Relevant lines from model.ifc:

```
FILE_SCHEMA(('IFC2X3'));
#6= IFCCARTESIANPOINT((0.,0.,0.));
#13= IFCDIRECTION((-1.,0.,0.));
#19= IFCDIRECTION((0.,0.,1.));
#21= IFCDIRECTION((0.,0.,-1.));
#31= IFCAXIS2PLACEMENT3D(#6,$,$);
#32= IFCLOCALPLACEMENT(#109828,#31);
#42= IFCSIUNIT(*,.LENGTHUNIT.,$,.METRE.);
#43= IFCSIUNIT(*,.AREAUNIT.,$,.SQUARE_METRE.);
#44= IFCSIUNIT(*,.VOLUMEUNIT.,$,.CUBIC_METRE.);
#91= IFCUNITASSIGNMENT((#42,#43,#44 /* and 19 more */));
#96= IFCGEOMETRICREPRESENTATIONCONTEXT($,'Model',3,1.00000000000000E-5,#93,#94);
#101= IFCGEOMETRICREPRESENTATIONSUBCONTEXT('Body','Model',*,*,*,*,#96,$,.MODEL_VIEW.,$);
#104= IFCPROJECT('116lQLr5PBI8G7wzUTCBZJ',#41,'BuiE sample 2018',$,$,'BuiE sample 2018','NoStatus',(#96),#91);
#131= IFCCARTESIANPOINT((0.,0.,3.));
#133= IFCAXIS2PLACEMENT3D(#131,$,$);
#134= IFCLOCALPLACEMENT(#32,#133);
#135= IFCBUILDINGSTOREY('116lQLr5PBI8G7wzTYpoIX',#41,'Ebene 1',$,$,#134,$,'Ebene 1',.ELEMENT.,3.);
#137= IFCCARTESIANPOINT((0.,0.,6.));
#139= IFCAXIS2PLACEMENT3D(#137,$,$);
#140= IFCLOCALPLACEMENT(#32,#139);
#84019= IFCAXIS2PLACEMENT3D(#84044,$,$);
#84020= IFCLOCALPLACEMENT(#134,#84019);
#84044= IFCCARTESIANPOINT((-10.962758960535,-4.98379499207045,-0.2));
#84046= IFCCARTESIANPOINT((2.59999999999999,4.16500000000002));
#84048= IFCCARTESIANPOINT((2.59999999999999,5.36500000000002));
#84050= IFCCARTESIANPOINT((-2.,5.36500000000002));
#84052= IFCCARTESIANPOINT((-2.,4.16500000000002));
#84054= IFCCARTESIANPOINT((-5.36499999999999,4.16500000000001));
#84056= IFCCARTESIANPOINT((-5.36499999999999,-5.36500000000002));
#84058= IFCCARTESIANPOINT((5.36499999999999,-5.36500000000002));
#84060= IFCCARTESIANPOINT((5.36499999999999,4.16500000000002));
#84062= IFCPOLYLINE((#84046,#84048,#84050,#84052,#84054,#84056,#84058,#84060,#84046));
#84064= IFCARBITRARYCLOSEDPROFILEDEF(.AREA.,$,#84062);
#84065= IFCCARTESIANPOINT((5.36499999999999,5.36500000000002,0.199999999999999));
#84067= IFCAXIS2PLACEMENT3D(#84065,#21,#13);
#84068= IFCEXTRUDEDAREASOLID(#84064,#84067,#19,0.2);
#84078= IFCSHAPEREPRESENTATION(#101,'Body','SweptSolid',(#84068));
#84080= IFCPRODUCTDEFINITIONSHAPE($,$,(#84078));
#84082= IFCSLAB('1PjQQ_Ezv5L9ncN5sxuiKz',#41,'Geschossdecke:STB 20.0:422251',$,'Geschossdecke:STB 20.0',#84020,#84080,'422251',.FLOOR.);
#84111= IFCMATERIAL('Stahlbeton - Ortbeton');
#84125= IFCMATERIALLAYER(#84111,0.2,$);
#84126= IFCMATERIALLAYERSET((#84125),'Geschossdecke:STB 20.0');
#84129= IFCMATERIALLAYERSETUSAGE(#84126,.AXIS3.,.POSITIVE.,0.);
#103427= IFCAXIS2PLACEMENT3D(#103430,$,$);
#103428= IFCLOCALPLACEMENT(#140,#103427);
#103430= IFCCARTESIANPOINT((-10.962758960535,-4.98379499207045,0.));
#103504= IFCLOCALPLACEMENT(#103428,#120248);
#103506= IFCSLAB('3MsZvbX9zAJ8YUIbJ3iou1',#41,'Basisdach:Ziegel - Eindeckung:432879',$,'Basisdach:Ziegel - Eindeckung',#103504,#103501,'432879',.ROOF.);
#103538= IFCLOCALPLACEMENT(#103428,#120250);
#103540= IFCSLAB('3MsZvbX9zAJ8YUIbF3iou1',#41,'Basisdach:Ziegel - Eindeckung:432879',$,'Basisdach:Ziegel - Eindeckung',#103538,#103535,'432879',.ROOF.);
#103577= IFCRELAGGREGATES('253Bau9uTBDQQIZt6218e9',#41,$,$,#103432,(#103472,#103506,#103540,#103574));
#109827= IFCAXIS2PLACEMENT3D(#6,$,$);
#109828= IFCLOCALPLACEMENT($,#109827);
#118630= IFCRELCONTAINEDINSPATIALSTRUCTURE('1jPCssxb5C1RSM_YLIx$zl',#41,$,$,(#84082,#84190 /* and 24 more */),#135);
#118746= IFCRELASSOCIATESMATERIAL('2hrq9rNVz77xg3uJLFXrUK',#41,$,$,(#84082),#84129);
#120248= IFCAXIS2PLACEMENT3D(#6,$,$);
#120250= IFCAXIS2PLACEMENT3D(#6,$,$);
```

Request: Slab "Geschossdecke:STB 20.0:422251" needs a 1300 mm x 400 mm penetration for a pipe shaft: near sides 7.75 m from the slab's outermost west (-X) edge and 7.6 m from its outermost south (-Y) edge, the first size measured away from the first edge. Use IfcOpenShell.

```python
import numpy as np
import ifcopenshell
import ifcopenshell.api.feature
import ifcopenshell.api.geometry
import ifcopenshell.api.root
import ifcopenshell.geom
import ifcopenshell.util.placement
import ifcopenshell.util.representation
import ifcopenshell.util.shape
import ifcopenshell.util.unit

model = ifcopenshell.open("model.ifc")
unit_scale = ifcopenshell.util.unit.calculate_unit_scale(model)
settings = ifcopenshell.geom.settings()


def volume(element):
    """Net volume in cubic metres, openings subtracted."""
    shape = ifcopenshell.geom.create_shape(settings, element)
    return ifcopenshell.util.shape.get_volume(shape.geometry)


slab = model.by_id(84082)
before = volume(slab)

# Extent in the slab's own axes, in metres. The edges named are its -X and -Y sides.
slab_shape = ifcopenshell.geom.create_shape(settings, slab)
vertices = ifcopenshell.util.shape.get_vertices(slab_shape.geometry)
x_min, y_min, bottom = vertices.min(axis=0)
top = vertices[:, 2].max()

opening = ifcopenshell.api.root.create_entity(model, ifc_class="IfcOpeningElement", name="Pipe shaft opening")
context = ifcopenshell.util.representation.get_context(model, "Model", "Body", "MODEL_VIEW")
width, depth = 1.3, 0.4
outline = [(0.0, 0.0), (width, 0.0), (width, depth), (0.0, depth), (0.0, 0.0)]
# Overshoot both faces by 50 mm so the cut is clean.
shape = ifcopenshell.api.geometry.add_slab_representation(
    model, context=context, depth=top - bottom + 0.1, polyline=outline
)
ifcopenshell.api.geometry.assign_representation(model, product=opening, representation=shape)

matrix = ifcopenshell.util.placement.get_local_placement(slab.ObjectPlacement)
matrix[:, 3] = matrix @ np.append(np.array([x_min + 7.75, y_min + 7.6, bottom - 0.05]) / unit_scale, 1.0)
ifcopenshell.api.geometry.edit_object_placement(model, product=opening, matrix=matrix, is_si=False)
ifcopenshell.api.feature.add_feature(model, feature=opening, element=slab)

after = volume(slab)

print(f"slab volume {before:.3f} -> {after:.3f} m3")

model.write("model_rev.ifc")
```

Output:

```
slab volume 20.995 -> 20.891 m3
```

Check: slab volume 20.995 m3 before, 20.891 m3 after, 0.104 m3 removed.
